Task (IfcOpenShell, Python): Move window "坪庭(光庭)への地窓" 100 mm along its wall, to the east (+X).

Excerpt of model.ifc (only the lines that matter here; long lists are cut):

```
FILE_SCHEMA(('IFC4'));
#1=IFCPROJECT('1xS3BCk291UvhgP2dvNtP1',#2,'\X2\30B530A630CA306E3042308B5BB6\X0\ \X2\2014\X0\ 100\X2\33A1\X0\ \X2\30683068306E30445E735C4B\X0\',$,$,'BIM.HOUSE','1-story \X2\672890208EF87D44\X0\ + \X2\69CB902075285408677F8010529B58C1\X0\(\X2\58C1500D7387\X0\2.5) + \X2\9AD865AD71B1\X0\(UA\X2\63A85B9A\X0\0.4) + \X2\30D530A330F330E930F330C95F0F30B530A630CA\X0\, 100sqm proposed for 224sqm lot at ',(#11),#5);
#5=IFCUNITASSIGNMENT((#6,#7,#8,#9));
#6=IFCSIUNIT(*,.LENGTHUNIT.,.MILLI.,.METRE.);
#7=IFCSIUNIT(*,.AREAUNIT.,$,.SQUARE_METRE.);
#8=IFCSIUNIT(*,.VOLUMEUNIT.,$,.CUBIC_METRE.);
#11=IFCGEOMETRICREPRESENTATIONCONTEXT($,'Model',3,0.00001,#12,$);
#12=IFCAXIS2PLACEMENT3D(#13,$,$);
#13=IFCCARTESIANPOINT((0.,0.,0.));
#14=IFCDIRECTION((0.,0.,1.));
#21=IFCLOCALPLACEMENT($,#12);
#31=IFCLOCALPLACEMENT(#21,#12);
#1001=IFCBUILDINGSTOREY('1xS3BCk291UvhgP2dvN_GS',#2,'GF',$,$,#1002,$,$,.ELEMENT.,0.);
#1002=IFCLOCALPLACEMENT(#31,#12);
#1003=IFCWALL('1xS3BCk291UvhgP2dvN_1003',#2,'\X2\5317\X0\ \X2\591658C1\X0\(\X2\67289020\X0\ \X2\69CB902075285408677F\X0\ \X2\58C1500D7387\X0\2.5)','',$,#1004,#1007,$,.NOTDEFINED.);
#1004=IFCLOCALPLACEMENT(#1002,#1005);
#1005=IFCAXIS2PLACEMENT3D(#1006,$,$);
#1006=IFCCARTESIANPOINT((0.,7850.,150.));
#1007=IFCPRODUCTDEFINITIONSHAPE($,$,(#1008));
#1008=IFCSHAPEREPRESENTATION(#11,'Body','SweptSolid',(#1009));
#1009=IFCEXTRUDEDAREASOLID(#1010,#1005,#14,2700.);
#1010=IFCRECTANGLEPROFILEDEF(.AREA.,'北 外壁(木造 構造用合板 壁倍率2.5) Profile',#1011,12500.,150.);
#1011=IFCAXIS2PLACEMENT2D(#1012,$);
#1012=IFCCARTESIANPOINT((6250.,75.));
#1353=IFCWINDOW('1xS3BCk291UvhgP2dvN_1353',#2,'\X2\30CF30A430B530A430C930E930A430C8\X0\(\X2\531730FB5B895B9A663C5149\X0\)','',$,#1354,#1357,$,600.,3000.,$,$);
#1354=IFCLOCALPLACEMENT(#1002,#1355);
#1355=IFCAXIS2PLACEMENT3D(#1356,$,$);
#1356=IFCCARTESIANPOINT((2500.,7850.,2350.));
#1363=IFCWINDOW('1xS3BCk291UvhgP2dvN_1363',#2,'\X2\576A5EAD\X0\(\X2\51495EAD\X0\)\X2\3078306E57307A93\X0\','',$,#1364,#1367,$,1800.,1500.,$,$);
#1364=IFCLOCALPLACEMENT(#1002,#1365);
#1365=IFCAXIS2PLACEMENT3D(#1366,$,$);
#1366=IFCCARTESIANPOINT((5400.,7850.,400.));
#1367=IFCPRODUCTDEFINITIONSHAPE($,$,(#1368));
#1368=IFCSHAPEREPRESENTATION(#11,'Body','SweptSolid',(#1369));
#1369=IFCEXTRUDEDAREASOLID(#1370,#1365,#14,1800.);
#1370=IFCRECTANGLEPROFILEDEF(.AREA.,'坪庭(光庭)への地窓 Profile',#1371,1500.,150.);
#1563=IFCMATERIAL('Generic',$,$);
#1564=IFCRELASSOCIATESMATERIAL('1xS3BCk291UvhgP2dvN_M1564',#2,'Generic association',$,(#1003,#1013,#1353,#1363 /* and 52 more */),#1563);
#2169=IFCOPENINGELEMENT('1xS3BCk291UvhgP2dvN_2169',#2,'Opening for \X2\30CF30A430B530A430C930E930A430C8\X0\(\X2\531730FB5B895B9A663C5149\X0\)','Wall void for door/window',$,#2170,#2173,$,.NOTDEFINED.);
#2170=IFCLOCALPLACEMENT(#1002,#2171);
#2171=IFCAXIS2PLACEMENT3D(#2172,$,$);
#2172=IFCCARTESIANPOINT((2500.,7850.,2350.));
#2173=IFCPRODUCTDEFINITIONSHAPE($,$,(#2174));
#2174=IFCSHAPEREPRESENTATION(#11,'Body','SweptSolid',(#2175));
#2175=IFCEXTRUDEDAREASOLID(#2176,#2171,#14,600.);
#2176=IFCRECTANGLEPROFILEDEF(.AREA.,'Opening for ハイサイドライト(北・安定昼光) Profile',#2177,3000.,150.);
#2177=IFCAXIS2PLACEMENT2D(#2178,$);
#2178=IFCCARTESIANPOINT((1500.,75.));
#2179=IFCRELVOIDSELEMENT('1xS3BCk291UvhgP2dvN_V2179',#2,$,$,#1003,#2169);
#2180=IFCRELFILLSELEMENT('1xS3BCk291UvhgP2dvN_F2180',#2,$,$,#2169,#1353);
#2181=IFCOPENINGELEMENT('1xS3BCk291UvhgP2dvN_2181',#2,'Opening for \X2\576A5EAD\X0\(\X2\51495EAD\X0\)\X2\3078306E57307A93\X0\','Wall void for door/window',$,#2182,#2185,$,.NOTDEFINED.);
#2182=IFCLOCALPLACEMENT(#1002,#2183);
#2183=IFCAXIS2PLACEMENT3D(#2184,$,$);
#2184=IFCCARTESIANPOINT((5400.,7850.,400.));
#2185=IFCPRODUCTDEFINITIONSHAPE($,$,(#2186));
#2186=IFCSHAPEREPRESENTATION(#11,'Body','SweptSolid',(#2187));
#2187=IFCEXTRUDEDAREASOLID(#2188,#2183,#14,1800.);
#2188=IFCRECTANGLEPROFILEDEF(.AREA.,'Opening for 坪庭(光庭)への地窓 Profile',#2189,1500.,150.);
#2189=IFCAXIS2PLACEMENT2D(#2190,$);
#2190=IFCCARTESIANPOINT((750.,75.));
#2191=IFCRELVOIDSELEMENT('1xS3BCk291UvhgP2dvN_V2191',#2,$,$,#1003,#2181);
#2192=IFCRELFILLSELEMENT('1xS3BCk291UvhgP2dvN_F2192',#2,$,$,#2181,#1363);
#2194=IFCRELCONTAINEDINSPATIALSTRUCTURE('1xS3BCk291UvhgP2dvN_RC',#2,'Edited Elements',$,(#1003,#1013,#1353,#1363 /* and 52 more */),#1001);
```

```python
import ifcopenshell
import ifcopenshell.api.geometry
import ifcopenshell.util.placement
import ifcopenshell.util.unit

model = ifcopenshell.open("model.ifc")
unit_scale = ifcopenshell.util.unit.calculate_unit_scale(model)

window = model.by_guid("1xS3BCk291UvhgP2dvN_1363")
opening = window.FillsVoids[0].RelatingOpeningElement
wall = opening.VoidsElements[0].RelatingBuildingElement

wall_matrix = ifcopenshell.util.placement.get_local_placement(wall.ObjectPlacement)
shift = wall_matrix[:3, 0] * 0.1 / unit_scale
before = ifcopenshell.util.placement.get_local_placement(window.ObjectPlacement)[:3, 3].copy()

# The window is not placed relative to its opening, so move both.
for product in (opening, window):
    matrix = ifcopenshell.util.placement.get_local_placement(product.ObjectPlacement)
    matrix[:3, 3] += shift
    ifcopenshell.api.geometry.edit_object_placement(model, product=product, matrix=matrix, is_si=False)

after = ifcopenshell.util.placement.get_local_placement(window.ObjectPlacement)[:3, 3]
print("window moved by", (after - before).round(3) + 0.0)

model.write("model_edited.ifc")
```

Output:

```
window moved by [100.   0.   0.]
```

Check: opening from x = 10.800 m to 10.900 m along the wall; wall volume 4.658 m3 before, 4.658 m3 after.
